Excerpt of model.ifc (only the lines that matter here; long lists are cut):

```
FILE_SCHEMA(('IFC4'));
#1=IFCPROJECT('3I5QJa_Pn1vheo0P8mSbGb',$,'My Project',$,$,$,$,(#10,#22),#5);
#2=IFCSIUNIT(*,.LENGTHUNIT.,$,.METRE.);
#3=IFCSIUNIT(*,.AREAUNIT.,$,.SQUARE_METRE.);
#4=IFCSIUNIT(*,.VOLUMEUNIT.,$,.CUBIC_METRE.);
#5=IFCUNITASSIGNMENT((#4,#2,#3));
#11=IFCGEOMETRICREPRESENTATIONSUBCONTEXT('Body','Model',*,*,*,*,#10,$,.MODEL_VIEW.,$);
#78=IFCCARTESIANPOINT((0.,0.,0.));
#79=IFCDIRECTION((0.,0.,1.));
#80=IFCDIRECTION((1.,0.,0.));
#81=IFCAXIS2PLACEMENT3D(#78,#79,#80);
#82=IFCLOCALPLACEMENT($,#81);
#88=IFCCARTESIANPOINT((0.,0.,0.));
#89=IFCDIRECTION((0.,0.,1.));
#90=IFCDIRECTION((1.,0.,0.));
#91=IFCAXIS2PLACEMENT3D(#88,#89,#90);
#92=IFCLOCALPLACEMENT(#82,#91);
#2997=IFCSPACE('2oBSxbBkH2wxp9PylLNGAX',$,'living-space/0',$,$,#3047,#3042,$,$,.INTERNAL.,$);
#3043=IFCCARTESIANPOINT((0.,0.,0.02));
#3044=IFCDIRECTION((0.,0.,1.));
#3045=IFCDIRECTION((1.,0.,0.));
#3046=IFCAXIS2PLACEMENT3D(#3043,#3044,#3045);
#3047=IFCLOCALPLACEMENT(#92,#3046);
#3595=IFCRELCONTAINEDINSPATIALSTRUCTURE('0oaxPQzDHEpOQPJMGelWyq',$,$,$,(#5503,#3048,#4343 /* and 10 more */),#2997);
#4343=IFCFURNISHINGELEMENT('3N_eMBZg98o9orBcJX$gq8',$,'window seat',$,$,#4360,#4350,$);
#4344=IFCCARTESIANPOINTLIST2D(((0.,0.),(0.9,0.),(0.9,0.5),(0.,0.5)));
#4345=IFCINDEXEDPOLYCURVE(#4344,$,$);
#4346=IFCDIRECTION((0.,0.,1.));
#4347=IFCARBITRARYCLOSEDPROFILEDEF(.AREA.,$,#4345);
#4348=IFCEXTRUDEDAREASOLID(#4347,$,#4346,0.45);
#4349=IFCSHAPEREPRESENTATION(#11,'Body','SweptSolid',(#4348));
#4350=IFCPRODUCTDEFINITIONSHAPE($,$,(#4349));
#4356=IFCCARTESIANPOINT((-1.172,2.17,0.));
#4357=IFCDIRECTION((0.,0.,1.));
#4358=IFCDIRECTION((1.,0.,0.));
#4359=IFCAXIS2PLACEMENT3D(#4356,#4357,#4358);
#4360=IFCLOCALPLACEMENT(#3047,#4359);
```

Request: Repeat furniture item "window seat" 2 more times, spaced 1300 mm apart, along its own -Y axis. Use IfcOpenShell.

```python
import ifcopenshell
import ifcopenshell.api.geometry
import ifcopenshell.api.root
import ifcopenshell.util.element
import ifcopenshell.util.placement

model = ifcopenshell.open("model.ifc")

source = model.by_guid("3N_eMBZg98o9orBcJX$gq8")
base = ifcopenshell.util.placement.get_local_placement(source.ObjectPlacement)
step = -base[:3, 1] * 1.3

for i in range(1, 3):
    copy = ifcopenshell.api.root.copy_class(model, product=source)
    copy.Representation = ifcopenshell.util.element.copy_deep(
        model, source.Representation, exclude=["IfcGeometricRepresentationContext", "IfcRepresentationMap"]
    )
    matrix = base.copy()
    matrix[:3, 3] += i * step
    print("added at", matrix[:3, 3].round(3) + 0.0)
    ifcopenshell.api.geometry.edit_object_placement(model, product=copy, matrix=matrix, is_si=False)

model.write("model_updated.ifc")
```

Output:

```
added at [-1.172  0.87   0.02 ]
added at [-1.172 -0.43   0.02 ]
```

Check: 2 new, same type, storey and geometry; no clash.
